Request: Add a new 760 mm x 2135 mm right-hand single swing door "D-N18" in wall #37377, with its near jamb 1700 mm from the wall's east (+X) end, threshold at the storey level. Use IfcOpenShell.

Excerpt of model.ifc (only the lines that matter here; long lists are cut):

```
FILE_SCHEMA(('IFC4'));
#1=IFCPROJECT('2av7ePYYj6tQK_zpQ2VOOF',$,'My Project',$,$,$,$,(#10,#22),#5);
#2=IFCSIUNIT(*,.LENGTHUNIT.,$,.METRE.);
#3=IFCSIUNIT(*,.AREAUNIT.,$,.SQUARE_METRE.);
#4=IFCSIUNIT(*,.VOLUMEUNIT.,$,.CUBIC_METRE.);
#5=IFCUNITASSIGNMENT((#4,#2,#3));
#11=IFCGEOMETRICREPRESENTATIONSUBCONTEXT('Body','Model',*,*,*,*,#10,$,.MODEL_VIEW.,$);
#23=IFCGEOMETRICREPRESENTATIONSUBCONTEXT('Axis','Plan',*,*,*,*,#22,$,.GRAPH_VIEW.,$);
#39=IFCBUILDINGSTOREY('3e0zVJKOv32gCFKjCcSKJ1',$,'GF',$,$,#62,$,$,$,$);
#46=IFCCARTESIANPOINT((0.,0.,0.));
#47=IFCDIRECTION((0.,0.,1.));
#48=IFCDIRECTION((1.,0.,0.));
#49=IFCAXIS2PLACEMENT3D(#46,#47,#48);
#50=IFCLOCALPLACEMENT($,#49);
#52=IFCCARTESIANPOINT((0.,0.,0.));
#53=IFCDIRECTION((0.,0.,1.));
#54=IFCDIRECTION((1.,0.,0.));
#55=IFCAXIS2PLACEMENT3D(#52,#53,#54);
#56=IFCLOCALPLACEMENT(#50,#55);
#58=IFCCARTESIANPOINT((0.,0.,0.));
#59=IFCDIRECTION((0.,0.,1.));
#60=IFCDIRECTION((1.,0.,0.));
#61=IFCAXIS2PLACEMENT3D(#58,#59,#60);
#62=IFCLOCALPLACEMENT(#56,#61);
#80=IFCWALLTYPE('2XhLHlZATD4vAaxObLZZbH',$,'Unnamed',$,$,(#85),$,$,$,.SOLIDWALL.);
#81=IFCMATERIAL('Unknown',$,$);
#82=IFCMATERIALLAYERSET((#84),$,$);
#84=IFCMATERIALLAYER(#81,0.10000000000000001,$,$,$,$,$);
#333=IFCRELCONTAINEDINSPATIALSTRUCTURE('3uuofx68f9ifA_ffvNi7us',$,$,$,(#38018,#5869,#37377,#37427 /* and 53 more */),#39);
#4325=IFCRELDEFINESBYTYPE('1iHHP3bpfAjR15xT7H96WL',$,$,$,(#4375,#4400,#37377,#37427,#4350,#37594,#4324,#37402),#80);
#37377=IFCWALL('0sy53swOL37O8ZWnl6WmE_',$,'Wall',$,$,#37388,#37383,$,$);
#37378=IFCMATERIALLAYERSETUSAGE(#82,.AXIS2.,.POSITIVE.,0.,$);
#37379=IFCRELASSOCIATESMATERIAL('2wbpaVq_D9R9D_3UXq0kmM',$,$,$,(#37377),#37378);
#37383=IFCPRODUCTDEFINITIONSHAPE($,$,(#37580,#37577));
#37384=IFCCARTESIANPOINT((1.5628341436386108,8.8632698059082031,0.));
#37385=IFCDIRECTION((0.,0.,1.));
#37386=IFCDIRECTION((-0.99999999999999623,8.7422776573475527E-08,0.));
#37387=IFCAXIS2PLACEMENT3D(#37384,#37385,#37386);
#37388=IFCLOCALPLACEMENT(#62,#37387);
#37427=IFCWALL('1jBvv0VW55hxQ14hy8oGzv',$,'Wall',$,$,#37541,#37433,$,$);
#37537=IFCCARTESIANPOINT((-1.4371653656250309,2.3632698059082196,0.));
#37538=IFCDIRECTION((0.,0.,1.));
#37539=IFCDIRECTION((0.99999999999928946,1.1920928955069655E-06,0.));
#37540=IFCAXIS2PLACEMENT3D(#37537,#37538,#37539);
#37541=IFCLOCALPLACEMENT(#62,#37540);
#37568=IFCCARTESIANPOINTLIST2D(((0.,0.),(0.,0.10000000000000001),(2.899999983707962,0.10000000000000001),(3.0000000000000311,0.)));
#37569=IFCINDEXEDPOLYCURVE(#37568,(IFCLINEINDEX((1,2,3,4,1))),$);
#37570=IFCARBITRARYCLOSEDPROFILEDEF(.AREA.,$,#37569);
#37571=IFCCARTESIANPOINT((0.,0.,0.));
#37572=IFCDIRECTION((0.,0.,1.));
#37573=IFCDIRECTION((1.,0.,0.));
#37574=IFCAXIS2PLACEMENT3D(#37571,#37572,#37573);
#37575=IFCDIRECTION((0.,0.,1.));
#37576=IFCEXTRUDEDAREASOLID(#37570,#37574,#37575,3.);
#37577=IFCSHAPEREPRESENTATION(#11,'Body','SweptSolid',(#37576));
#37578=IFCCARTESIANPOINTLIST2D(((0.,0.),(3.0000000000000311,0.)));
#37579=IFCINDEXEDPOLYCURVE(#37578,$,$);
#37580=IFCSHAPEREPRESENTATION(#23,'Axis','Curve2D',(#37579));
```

```python
import numpy as np
import ifcopenshell
import ifcopenshell.api.feature
import ifcopenshell.api.geometry
import ifcopenshell.api.root
import ifcopenshell.api.spatial
import ifcopenshell.geom
import ifcopenshell.util.element
import ifcopenshell.util.placement
import ifcopenshell.util.representation
import ifcopenshell.util.shape
import ifcopenshell.util.unit

model = ifcopenshell.open("model.ifc")
unit_scale = ifcopenshell.util.unit.calculate_unit_scale(model)
settings = ifcopenshell.geom.settings()


def volume(element):
    """Net volume in cubic metres, openings subtracted."""
    shape = ifcopenshell.geom.create_shape(settings, element)
    return ifcopenshell.util.shape.get_volume(shape.geometry)


wall = model.by_id(37377)
storey = ifcopenshell.util.element.get_container(wall, ifc_class="IfcBuildingStorey")
context = ifcopenshell.util.representation.get_context(model, "Model", "Body", "MODEL_VIEW")
before = volume(wall)

width, height, from_end, sill = 0.76, 2.135, 1.7, 0.0  # metres

# The wall runs along its own X axis, and the end named is its -X end.
wall_shape = ifcopenshell.geom.create_shape(settings, wall)
x, y, z = ifcopenshell.util.shape.get_vertices(wall_shape.geometry).T
start = x.min() + from_end
face, thickness = float(y.min()), float(y.max() - y.min())
wall_matrix = ifcopenshell.util.placement.get_local_placement(wall.ObjectPlacement)
level = ifcopenshell.util.placement.get_local_placement(storey.ObjectPlacement)[2, 3]


def in_wall(x, y):
    """Placement at x, y metres in the wall's axes, at sill height."""
    matrix = wall_matrix.copy()
    matrix[:, 3] = wall_matrix @ np.array([x / unit_scale, y / unit_scale, 0.0, 1.0])
    matrix[2, 3] = level + sill / unit_scale
    return matrix


# Opening: a box that overshoots both wall faces by 50 mm.
opening = ifcopenshell.api.root.create_entity(model, ifc_class="IfcOpeningElement", predefined_type="OPENING")
box = ifcopenshell.api.geometry.add_wall_representation(
    model, context=context, length=width, height=height, thickness=thickness + 0.1
)
ifcopenshell.api.geometry.assign_representation(model, product=opening, representation=box)
ifcopenshell.api.geometry.edit_object_placement(model, product=opening, matrix=in_wall(start, face - 0.05), is_si=False)
ifcopenshell.api.feature.add_feature(model, feature=opening, element=wall)

door = ifcopenshell.api.root.create_entity(model, ifc_class="IfcDoor", name="D-N18", predefined_type="DOOR")
door.OverallWidth, door.OverallHeight = width / unit_scale, height / unit_scale
door.OperationType = "SINGLE_SWING_RIGHT"
body = ifcopenshell.api.geometry.add_door_representation(
    model,
    context=context,
    overall_width=door.OverallWidth,
    overall_height=door.OverallHeight,
    operation_type="SINGLE_SWING_RIGHT",
    lining_properties={"LiningDepth": thickness / unit_scale, "ThresholdDepth": thickness / unit_scale},
)
ifcopenshell.api.geometry.assign_representation(model, product=door, representation=body)
ifcopenshell.api.spatial.assign_container(model, products=[door], relating_structure=storey)
ifcopenshell.api.feature.add_filling(model, opening=opening, element=door)

# The lining spans the wall, so the door starts at the wall face.
ifcopenshell.api.geometry.edit_object_placement(model, product=door, matrix=in_wall(start, face), is_si=False)

after = volume(wall)

print(f"wall volume {before:.3f} -> {after:.3f} m3")

model.write("model_v2.ifc")
```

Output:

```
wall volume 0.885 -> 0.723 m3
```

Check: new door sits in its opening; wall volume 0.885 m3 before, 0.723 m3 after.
